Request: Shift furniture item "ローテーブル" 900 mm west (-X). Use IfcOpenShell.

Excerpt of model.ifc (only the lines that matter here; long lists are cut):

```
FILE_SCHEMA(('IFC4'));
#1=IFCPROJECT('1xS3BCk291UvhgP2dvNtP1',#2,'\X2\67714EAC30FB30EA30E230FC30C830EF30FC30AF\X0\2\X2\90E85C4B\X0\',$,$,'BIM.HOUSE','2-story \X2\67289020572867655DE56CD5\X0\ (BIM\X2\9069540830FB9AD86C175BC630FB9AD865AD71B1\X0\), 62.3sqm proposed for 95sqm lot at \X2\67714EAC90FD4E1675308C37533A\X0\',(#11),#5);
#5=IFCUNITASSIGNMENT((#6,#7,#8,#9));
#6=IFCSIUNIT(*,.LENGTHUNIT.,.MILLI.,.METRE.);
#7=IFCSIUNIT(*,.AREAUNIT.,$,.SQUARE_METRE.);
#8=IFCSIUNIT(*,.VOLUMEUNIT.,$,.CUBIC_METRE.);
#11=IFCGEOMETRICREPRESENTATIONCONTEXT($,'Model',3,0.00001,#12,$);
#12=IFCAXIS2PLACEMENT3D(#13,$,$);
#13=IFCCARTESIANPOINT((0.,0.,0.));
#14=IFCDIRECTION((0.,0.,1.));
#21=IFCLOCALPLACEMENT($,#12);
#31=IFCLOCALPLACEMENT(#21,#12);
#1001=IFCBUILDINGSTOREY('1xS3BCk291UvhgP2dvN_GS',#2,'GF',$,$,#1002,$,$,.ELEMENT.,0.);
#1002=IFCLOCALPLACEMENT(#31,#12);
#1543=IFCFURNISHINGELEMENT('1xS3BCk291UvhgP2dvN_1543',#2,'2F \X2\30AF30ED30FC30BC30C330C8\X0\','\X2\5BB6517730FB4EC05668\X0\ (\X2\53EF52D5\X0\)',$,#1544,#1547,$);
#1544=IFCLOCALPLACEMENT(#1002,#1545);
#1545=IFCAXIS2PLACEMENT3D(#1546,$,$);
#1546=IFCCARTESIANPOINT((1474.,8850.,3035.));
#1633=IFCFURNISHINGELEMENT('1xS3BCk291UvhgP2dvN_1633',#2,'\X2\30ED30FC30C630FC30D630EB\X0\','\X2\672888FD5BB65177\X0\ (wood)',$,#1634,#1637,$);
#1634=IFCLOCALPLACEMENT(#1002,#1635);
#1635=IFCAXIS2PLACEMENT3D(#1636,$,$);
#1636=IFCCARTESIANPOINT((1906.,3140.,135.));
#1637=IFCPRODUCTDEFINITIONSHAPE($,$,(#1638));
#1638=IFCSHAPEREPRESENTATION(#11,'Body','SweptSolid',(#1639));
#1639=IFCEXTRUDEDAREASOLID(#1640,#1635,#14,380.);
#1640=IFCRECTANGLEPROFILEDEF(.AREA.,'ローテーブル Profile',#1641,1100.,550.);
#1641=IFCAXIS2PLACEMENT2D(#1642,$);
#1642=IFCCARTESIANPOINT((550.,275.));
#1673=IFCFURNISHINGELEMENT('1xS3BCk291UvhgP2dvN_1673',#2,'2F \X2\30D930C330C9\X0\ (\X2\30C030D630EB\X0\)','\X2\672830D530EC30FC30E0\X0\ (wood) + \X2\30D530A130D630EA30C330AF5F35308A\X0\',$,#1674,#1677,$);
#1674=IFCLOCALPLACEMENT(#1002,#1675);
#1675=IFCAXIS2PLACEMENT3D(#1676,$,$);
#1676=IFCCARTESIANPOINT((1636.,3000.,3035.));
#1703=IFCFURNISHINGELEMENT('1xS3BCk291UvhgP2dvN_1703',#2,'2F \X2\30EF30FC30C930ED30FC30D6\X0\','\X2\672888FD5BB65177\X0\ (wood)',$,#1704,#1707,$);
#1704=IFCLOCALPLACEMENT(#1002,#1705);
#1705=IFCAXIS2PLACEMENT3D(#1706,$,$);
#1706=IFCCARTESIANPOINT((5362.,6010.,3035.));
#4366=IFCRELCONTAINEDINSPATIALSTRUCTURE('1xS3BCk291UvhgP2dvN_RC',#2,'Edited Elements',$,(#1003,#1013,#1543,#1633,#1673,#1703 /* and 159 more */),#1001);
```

```python
import ifcopenshell
import ifcopenshell.api.geometry
import ifcopenshell.util.placement

model = ifcopenshell.open("model.ifc")

item = model.by_guid("1xS3BCk291UvhgP2dvN_1633")
matrix = ifcopenshell.util.placement.get_local_placement(item.ObjectPlacement)
matrix[0, 3] -= 900.0
ifcopenshell.api.geometry.edit_object_placement(model, product=item, matrix=matrix, is_si=False)

print(ifcopenshell.util.placement.get_local_placement(item.ObjectPlacement).round(3) + 0.0)

model.write("model_rev.ifc")
```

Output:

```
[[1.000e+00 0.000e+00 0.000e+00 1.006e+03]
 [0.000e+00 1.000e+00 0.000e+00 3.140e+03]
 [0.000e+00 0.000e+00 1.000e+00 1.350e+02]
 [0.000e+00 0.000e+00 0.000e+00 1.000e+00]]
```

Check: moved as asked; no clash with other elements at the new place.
